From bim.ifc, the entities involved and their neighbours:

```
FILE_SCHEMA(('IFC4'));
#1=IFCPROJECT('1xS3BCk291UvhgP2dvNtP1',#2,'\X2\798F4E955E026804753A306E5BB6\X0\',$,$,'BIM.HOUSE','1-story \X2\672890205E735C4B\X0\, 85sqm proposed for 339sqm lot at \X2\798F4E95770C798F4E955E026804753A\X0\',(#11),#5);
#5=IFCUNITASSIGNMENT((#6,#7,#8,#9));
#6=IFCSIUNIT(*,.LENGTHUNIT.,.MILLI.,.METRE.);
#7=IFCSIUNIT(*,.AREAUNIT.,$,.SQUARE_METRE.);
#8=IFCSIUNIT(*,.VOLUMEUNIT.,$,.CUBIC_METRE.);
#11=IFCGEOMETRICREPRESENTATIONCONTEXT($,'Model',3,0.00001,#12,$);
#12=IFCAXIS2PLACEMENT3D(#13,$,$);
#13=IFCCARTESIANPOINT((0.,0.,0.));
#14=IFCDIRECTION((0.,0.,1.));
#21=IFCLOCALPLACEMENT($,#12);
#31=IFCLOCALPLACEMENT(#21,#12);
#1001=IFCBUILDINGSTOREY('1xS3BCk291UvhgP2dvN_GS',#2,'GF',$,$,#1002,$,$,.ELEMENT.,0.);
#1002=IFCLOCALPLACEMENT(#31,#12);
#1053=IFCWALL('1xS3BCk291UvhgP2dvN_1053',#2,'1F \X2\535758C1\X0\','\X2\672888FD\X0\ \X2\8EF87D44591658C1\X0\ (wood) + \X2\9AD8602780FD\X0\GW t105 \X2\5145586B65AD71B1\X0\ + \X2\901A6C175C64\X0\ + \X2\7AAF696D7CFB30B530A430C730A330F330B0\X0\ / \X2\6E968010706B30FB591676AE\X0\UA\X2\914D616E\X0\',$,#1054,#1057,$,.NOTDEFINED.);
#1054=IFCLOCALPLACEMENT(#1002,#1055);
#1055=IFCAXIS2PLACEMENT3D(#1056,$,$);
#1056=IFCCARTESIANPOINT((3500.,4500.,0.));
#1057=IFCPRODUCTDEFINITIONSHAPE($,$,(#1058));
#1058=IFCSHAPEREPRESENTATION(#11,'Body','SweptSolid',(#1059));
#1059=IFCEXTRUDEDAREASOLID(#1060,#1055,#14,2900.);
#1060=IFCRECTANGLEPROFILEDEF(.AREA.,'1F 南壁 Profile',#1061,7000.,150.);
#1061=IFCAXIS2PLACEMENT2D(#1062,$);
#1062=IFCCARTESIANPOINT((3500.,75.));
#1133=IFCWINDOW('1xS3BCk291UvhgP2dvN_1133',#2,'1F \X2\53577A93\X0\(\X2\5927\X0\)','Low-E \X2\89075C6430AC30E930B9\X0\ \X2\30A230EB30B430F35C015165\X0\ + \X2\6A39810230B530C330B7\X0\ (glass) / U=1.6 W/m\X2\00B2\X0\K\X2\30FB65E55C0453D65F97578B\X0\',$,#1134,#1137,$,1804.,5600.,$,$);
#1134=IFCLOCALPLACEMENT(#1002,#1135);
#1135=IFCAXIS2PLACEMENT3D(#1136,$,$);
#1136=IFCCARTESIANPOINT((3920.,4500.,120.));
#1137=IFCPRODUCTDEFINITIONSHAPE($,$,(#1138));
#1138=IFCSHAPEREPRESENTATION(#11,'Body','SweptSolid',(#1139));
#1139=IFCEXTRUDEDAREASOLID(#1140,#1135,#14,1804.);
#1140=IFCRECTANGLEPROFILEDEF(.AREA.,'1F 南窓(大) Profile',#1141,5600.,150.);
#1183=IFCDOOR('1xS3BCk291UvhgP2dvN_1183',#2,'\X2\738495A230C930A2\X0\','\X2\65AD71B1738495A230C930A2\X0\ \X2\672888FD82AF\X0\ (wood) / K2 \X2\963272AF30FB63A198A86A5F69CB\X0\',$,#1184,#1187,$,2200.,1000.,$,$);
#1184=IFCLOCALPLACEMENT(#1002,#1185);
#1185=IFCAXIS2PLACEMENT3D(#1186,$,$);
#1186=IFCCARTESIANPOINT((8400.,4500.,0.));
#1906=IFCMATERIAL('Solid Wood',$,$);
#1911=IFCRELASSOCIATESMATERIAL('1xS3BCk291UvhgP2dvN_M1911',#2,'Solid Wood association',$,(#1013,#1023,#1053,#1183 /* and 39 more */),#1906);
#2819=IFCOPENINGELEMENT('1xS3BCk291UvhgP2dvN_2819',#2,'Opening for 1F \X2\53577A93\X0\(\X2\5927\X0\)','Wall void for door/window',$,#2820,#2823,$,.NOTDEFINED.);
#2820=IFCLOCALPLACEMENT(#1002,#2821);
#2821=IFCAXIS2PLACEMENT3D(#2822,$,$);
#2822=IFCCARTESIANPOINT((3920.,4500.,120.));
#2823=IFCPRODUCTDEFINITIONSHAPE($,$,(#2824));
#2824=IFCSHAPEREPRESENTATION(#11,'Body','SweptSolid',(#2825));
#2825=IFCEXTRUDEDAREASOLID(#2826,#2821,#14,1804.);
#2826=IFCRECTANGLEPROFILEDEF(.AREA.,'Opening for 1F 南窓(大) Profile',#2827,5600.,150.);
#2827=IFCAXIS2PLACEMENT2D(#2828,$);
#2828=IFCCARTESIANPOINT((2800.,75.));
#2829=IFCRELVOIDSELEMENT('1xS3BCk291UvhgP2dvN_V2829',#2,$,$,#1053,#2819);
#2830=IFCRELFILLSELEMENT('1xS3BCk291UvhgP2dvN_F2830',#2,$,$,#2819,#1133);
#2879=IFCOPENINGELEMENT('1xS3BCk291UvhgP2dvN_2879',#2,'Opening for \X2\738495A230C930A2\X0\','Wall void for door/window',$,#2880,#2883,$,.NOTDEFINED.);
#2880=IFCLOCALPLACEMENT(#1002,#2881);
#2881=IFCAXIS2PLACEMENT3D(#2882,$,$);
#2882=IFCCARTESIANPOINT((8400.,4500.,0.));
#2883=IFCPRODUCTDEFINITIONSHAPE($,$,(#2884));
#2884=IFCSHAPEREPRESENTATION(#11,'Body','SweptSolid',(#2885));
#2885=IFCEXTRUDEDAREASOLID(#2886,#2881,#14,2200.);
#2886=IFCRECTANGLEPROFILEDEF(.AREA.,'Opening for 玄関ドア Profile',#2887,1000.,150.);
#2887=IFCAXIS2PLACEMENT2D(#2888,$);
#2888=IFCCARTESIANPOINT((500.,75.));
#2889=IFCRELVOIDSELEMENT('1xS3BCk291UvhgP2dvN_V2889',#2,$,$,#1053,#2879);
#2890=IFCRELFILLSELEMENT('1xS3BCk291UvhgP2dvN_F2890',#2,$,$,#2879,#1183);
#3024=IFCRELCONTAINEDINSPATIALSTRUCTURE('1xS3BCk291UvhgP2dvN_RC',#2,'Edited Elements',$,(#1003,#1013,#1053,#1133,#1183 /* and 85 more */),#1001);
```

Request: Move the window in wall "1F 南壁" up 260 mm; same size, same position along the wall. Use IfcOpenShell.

```python
import numpy as np
import ifcopenshell
import ifcopenshell.api.geometry
import ifcopenshell.util.placement
import ifcopenshell.util.unit

model = ifcopenshell.open("bim.ifc")
unit_scale = ifcopenshell.util.unit.calculate_unit_scale(model)

window = model.by_guid("1xS3BCk291UvhgP2dvN_1133")
opening = window.FillsVoids[0].RelatingOpeningElement
dz = 0.26 / unit_scale

shift = np.array([0.0, 0.0, dz])
# The window is not placed relative to its opening, so move both.
for product in (opening, window):
    matrix = ifcopenshell.util.placement.get_local_placement(product.ObjectPlacement)
    matrix[:3, 3] += shift
    ifcopenshell.api.geometry.edit_object_placement(model, product=product, matrix=matrix, is_si=False)

print(f"moved by {dz * unit_scale:+.3f} m")

model.write("bim_updated.ifc")
```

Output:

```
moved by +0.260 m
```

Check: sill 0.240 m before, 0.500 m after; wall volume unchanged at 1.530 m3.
